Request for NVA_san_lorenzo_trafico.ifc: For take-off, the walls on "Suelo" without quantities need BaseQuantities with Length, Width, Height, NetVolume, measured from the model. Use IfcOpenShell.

First a look at what the model holds.

```python
import ifcopenshell
import ifcopenshell.util.element
import ifcopenshell.util.unit

model = ifcopenshell.open("NVA_san_lorenzo_trafico.ifc")
print(model.schema)
for unit_type in ("LENGTHUNIT", "AREAUNIT", "VOLUMEUNIT"):
    print(unit_type, ifcopenshell.util.unit.calculate_unit_scale(model, unit_type))
storey = next(s for s in model.by_type("IfcBuildingStorey") if s.Name == "Suelo")
walls = [e for e in ifcopenshell.util.element.get_decomposition(storey) if e.is_a("IfcWall")]
for e in sorted(walls, key=lambda e: e.id()):
    print(e.id(), e.is_a(), e.Name, list(ifcopenshell.util.element.get_psets(e, qtos_only=True)), sep=" | ")
```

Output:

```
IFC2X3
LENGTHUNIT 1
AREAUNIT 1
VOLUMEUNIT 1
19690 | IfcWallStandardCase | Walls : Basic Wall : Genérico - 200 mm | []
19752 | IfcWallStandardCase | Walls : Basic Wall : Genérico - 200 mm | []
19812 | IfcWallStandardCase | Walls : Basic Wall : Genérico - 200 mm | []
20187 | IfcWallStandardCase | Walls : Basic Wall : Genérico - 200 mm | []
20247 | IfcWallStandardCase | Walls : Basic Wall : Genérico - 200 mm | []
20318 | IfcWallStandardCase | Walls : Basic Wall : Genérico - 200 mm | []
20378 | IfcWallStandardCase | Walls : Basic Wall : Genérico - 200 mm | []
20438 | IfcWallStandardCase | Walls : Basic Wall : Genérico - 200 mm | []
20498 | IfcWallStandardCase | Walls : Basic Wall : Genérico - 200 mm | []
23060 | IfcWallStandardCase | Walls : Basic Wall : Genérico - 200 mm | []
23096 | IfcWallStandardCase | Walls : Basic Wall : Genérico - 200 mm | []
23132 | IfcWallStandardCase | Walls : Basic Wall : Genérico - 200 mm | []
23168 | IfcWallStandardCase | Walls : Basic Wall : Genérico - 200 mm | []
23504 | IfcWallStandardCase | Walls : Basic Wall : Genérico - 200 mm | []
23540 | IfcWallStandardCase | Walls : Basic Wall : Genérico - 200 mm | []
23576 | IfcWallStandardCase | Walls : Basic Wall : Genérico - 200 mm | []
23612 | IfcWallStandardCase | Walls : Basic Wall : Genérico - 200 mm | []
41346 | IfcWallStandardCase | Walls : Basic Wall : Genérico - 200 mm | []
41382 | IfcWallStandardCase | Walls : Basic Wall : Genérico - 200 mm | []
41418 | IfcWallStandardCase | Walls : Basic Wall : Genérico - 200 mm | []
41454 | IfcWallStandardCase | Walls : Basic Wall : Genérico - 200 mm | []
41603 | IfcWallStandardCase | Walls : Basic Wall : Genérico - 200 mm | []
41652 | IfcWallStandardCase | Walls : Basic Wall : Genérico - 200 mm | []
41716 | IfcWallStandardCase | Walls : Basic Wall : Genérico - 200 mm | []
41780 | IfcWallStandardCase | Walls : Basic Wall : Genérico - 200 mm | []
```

```python
import ifcopenshell
import ifcopenshell.api.pset
import ifcopenshell.geom
import ifcopenshell.util.element
import ifcopenshell.util.shape
import ifcopenshell.util.unit

model = ifcopenshell.open("NVA_san_lorenzo_trafico.ifc")
unit_scale = ifcopenshell.util.unit.calculate_unit_scale(model)
volume_scale = ifcopenshell.util.unit.calculate_unit_scale(model, "VOLUMEUNIT")
settings = ifcopenshell.geom.settings()

storey = next(s for s in model.by_type("IfcBuildingStorey") if s.Name == "Suelo")
walls = [e for e in ifcopenshell.util.element.get_decomposition(storey) if e.is_a("IfcWall")]

for e in sorted(walls, key=lambda e: e.id()):
    if ifcopenshell.util.element.get_psets(e, qtos_only=True, should_inherit=False):
        continue
    # Geometry comes back in metres, in the element's own axes.
    shape = ifcopenshell.geom.create_shape(settings, e)
    values = {
        "Length": ifcopenshell.util.shape.get_x(shape.geometry) / unit_scale,
        "Width": ifcopenshell.util.shape.get_y(shape.geometry) / unit_scale,
        "Height": ifcopenshell.util.shape.get_z(shape.geometry) / unit_scale,
        "NetVolume": ifcopenshell.util.shape.get_volume(shape.geometry) / volume_scale,
    }
    qto = ifcopenshell.api.pset.add_qto(model, product=e, name="BaseQuantities")
    ifcopenshell.api.pset.edit_qto(model, qto=qto, properties=values)
    print(e.id(), {k: round(v, 3) for k, v in values.items()})

model.write("NVA_san_lorenzo_trafico-out.ifc")
```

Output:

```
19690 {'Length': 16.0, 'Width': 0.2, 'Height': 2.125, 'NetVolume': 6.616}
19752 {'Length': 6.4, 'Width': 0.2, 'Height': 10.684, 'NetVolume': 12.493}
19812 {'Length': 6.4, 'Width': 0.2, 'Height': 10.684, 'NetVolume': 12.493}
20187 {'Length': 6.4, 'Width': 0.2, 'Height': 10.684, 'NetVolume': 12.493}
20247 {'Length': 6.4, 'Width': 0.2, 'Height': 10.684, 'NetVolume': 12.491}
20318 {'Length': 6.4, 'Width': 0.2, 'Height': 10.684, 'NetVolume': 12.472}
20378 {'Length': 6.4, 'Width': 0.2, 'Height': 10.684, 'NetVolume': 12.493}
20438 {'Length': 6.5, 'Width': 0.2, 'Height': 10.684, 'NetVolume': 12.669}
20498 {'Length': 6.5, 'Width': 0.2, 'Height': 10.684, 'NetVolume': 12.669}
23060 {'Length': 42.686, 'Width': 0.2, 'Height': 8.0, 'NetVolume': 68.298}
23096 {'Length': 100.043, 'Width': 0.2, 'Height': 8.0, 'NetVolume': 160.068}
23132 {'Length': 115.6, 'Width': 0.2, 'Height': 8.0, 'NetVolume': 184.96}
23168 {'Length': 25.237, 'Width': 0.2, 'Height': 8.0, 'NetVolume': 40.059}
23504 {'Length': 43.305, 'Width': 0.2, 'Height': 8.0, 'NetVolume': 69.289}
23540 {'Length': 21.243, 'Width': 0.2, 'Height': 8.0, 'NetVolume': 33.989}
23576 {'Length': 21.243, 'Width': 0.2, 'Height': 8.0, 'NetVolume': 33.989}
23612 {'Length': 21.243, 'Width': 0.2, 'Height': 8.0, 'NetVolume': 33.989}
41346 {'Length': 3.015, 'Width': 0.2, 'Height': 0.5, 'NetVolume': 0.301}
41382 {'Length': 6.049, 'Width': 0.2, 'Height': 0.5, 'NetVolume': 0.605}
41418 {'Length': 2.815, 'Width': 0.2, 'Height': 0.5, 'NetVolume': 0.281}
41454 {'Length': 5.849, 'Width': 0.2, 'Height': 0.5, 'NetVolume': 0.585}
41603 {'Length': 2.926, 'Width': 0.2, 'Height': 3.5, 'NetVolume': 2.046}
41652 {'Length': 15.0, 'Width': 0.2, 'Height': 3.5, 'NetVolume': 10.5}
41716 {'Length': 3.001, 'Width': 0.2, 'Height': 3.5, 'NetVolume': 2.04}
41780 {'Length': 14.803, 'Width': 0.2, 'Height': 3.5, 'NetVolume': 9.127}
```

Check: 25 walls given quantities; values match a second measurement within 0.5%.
